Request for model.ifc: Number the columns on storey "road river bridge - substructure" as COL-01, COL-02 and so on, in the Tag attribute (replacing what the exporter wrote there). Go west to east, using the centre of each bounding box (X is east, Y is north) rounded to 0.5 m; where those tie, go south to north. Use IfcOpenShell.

First a look at what the model holds.

```python
import ifcopenshell
import ifcopenshell.util.element
import ifcopenshell.util.placement

model = ifcopenshell.open("model.ifc")
print(model.schema)
storey = next(s for s in model.by_type("IfcBuildingStorey") if s.Name == "road river bridge - substructure")
columns = [e for e in ifcopenshell.util.element.get_decomposition(storey) if e.is_a("IfcColumn")]
for e in sorted(columns, key=lambda e: e.id()):
    origin = ifcopenshell.util.placement.get_local_placement(e.ObjectPlacement)[:3, 3]
    print(e.id(), e.Tag, e.Name, origin.round(2) + 0.0, sep=" | ")
```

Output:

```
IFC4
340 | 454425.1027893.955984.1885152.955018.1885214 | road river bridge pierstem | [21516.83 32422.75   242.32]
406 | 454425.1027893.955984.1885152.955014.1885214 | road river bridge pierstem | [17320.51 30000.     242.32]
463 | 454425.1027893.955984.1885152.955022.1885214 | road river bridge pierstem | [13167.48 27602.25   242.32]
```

```python
import ifcopenshell
import ifcopenshell.geom
import ifcopenshell.util.element
import ifcopenshell.util.shape

model = ifcopenshell.open("model.ifc")
settings = ifcopenshell.geom.settings()
settings.set("use-world-coords", True)


def centre(element):
    shape = ifcopenshell.geom.create_shape(settings, element)
    return ifcopenshell.util.shape.get_bbox_centroid(shape.geometry)


storey = next(s for s in model.by_type("IfcBuildingStorey") if s.Name == "road river bridge - substructure")
columns = [e for e in ifcopenshell.util.element.get_decomposition(storey) if e.is_a("IfcColumn")]

# Insertion points can sit at a corner or the storey origin, so sort by the geometry (in metres).
centres = {e: centre(e) for e in columns}
columns.sort(key=lambda e: (round(centres[e][0] / 0.5), centres[e][1]))

for i, e in enumerate(columns, start=1):
    number = f"COL-{i:02d}"
    e.Tag = number
    print(e.id(), number)

model.write("model_edited.ifc")
```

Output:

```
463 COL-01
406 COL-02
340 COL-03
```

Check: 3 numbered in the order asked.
